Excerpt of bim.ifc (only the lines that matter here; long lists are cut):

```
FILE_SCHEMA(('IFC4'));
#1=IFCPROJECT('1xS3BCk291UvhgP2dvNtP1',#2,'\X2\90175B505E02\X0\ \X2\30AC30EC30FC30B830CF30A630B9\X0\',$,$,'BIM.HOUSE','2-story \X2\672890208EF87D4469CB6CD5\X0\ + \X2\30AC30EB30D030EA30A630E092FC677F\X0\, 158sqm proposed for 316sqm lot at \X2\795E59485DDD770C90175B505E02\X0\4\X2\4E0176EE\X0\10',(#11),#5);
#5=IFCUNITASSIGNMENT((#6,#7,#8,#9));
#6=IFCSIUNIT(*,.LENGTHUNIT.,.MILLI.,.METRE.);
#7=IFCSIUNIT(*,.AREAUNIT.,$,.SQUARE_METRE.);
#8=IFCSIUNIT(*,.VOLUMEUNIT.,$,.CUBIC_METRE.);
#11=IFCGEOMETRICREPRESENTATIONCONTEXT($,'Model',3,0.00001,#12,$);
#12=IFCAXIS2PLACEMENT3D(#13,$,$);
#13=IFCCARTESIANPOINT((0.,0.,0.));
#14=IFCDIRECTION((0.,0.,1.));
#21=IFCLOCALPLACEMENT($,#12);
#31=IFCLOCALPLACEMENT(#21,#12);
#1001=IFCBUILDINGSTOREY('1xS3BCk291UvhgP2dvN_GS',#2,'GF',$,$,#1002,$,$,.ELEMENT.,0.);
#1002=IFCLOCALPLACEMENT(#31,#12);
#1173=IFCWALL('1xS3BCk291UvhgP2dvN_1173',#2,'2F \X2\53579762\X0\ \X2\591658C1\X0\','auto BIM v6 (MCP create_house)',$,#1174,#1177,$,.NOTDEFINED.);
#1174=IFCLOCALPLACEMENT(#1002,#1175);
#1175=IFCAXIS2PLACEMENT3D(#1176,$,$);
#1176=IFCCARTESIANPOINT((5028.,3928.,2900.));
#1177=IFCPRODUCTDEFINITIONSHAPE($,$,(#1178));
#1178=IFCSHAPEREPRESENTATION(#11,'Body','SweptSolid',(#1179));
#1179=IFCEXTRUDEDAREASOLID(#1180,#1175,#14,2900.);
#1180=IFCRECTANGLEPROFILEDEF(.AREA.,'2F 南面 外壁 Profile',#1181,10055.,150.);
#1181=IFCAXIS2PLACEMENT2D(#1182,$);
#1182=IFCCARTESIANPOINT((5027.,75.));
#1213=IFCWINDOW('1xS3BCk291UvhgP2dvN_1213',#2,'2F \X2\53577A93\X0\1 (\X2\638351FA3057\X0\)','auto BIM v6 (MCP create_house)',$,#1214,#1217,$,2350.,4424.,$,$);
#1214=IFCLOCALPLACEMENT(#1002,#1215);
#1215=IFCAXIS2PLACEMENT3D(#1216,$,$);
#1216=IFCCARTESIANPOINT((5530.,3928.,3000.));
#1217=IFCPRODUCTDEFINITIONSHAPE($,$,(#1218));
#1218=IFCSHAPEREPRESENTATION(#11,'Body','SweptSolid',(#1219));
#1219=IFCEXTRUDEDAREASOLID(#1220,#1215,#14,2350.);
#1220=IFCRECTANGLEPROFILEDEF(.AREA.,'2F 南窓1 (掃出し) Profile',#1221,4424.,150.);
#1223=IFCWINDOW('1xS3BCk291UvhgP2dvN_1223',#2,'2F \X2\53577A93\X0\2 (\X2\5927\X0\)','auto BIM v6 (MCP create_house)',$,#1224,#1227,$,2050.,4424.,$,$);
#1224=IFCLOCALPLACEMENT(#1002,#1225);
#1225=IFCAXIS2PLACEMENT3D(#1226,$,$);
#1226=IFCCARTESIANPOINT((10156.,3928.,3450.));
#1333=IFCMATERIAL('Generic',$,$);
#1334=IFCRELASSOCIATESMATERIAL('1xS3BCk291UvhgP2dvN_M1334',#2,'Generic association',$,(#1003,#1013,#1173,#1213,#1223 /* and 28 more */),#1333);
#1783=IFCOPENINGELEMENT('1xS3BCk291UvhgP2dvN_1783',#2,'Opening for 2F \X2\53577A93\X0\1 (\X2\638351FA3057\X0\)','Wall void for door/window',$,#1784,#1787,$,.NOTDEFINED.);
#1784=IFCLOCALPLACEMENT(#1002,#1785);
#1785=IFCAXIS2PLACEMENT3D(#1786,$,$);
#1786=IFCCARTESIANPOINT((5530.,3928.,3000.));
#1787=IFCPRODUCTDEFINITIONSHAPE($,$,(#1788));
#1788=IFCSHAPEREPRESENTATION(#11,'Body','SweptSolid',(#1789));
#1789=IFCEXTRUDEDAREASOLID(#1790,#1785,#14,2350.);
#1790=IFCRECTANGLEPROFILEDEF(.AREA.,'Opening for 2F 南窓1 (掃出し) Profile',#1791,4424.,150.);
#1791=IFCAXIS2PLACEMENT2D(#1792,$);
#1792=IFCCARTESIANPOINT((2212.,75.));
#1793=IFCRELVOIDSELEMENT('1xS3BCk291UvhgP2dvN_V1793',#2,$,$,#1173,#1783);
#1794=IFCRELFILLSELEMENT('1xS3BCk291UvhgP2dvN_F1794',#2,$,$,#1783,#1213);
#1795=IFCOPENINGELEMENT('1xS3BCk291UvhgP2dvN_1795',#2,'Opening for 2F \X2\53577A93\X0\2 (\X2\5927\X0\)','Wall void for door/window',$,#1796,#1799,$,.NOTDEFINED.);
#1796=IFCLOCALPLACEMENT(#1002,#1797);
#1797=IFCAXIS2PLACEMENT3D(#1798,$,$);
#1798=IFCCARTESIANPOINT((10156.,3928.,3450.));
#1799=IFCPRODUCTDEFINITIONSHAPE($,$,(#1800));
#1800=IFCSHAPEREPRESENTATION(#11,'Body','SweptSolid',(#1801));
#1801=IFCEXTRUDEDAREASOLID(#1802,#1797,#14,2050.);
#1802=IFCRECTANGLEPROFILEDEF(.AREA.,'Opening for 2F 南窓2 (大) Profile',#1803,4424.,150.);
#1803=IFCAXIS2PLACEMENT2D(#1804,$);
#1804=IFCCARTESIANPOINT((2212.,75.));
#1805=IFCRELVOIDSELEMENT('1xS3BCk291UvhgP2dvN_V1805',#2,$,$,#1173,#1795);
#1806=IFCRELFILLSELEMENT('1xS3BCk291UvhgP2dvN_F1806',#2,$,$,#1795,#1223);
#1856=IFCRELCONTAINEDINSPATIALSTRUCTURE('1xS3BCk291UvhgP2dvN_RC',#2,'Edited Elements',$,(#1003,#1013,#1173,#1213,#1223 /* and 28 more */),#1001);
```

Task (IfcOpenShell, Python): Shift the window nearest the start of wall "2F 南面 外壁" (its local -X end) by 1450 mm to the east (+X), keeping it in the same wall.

```python
import ifcopenshell
import ifcopenshell.api.geometry
import ifcopenshell.util.placement

model = ifcopenshell.open("bim.ifc")

window = model.by_guid("1xS3BCk291UvhgP2dvN_1213")
opening = window.FillsVoids[0].RelatingOpeningElement
wall = opening.VoidsElements[0].RelatingBuildingElement

wall_matrix = ifcopenshell.util.placement.get_local_placement(wall.ObjectPlacement)
shift = wall_matrix[:3, 0] * 1450.0
before = ifcopenshell.util.placement.get_local_placement(window.ObjectPlacement)[:3, 3].copy()

# The window is not placed relative to its opening, so move both.
for product in (opening, window):
    matrix = ifcopenshell.util.placement.get_local_placement(product.ObjectPlacement)
    matrix[:3, 3] += shift
    ifcopenshell.api.geometry.edit_object_placement(model, product=product, matrix=matrix, is_si=False)

after = ifcopenshell.util.placement.get_local_placement(window.ObjectPlacement)[:3, 3]
print("window moved by", (after - before).round(3) + 0.0)

model.write("bim_v2.ifc")
```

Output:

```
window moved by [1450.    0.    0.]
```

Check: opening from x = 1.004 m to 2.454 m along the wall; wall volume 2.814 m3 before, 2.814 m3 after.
